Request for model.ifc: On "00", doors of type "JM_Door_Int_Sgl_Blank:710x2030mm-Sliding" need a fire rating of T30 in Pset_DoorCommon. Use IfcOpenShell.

First a look at what the model holds.

```python
import ifcopenshell
import ifcopenshell.util.element

model = ifcopenshell.open("model.ifc")
print(model.schema)
storey = next(s for s in model.by_type("IfcBuildingStorey") if s.Name == "00")
doors = [e for e in ifcopenshell.util.element.get_decomposition(storey) if e.is_a("IfcDoor")]
seen = {}
for e in doors:
    element_type = ifcopenshell.util.element.get_type(e)
    key = (element_type.Name if element_type != e and element_type else None, ifcopenshell.util.element.get_pset(e, "Pset_DoorCommon", "FireRating"))
    seen[key] = seen.get(key, 0) + 1
for (name, value), count in sorted(seen.items(), key=str):
    print(count, "x", name, "|", value)
```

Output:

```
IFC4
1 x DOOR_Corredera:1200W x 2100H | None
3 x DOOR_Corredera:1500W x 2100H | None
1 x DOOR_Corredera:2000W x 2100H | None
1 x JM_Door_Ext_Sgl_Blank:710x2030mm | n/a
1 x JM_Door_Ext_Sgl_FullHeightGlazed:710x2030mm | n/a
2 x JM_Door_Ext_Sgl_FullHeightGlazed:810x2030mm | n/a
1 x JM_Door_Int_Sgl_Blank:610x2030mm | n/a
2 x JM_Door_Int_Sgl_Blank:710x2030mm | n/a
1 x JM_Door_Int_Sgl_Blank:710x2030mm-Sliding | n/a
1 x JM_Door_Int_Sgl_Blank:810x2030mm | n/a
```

```python
import ifcopenshell
import ifcopenshell.api.pset
import ifcopenshell.util.element

model = ifcopenshell.open("model.ifc")

storey = next(s for s in model.by_type("IfcBuildingStorey") if s.Name == "00")
doors = [e for e in ifcopenshell.util.element.get_decomposition(storey) if e.is_a("IfcDoor")]

count = 0
for e in doors:
    element_type = ifcopenshell.util.element.get_type(e)
    if element_type in (None, e) or element_type.Name != "JM_Door_Int_Sgl_Blank:710x2030mm-Sliding":
        continue
    # add_pset returns the element's existing set when there is one.
    pset = ifcopenshell.api.pset.add_pset(model, product=e, name="Pset_DoorCommon")
    ifcopenshell.api.pset.edit_pset(model, pset=pset, properties={"FireRating": "T30"})
    count += 1

print(count, "doors updated")

model.write("model-out.ifc")
```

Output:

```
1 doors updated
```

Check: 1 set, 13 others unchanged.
